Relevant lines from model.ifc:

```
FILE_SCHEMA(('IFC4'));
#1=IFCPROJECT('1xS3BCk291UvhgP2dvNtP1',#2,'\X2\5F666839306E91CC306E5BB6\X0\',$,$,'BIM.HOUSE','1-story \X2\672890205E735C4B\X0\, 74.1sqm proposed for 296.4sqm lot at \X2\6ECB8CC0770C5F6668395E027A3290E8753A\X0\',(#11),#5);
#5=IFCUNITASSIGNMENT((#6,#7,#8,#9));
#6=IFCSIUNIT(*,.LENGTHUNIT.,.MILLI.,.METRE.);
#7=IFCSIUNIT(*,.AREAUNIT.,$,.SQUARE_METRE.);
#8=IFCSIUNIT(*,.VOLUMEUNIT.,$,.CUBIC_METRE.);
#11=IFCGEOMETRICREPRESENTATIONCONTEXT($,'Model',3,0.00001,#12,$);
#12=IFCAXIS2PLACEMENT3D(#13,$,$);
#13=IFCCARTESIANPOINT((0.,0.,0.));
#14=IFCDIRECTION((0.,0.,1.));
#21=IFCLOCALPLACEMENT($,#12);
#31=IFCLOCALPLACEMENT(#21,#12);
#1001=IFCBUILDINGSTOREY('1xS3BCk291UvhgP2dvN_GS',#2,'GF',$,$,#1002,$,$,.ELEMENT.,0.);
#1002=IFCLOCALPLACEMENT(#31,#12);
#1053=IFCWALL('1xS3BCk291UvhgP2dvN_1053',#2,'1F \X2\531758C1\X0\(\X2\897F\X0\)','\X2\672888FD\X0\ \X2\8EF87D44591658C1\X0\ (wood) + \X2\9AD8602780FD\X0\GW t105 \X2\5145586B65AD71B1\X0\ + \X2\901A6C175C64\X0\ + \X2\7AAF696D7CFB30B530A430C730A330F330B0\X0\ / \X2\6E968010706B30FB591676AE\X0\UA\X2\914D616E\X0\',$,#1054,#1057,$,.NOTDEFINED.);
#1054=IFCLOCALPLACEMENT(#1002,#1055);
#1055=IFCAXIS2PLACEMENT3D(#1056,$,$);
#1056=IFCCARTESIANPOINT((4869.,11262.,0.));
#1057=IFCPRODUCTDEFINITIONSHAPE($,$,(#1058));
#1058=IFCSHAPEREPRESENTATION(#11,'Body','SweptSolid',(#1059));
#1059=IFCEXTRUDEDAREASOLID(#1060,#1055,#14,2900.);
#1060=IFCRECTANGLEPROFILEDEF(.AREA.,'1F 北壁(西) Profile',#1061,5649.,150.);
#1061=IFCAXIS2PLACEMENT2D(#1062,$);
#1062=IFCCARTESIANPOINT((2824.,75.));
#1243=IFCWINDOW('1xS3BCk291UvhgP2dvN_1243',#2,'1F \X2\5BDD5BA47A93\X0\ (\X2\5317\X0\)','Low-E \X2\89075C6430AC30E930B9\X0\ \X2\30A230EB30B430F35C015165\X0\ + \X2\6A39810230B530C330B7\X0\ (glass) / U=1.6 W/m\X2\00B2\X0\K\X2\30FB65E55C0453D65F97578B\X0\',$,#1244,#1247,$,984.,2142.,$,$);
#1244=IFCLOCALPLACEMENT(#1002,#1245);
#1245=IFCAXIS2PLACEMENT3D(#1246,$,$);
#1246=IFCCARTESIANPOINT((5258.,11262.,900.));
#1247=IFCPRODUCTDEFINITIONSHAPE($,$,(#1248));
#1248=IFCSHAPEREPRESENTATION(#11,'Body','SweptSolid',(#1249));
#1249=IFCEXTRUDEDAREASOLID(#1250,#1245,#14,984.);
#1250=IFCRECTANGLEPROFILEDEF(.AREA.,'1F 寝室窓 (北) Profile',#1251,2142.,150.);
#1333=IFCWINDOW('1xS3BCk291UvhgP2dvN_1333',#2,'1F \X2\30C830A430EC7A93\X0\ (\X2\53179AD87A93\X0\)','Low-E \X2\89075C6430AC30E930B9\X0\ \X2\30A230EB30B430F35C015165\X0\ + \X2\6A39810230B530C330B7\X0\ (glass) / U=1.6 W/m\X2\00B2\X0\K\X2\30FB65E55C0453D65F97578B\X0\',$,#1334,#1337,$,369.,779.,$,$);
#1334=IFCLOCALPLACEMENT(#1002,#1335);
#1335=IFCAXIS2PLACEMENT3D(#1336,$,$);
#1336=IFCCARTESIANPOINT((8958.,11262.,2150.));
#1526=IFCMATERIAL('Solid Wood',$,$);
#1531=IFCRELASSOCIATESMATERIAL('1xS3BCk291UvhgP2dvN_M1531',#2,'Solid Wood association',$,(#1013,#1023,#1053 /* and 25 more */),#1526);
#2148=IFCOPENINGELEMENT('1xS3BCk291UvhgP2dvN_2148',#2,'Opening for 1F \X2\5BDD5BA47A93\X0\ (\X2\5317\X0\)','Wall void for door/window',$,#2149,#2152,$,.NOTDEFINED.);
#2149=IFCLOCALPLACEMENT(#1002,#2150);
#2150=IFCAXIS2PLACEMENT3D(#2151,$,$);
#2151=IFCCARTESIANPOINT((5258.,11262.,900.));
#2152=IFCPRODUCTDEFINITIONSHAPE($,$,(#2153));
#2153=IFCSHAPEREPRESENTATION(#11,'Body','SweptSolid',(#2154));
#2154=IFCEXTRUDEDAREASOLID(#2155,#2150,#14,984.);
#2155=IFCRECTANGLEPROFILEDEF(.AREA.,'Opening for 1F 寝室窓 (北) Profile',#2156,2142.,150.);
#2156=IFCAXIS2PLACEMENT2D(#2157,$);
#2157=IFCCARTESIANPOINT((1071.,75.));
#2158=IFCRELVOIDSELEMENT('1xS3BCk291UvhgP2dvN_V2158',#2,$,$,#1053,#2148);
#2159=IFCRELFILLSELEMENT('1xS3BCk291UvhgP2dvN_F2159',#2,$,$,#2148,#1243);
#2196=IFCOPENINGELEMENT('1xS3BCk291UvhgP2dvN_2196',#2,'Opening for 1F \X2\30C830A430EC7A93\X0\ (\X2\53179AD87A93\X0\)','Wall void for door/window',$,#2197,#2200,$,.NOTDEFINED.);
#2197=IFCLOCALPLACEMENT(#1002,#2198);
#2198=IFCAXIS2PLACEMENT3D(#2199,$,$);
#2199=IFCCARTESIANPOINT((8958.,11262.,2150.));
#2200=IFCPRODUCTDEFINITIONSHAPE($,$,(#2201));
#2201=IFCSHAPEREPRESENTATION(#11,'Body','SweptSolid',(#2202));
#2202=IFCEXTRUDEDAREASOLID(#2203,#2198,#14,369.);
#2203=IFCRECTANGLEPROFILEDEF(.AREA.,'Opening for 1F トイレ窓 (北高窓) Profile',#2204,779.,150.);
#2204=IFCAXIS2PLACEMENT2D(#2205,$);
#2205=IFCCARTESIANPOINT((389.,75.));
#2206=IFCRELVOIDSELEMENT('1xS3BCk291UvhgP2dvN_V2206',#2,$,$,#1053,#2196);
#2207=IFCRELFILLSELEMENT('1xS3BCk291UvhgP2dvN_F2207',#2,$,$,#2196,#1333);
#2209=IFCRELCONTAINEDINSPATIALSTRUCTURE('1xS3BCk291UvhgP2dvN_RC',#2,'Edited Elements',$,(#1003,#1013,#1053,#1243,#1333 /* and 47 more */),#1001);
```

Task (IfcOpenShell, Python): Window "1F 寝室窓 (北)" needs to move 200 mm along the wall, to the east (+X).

```python
import ifcopenshell
import ifcopenshell.api.geometry
import ifcopenshell.util.placement
import ifcopenshell.util.unit

model = ifcopenshell.open("model.ifc")
unit_scale = ifcopenshell.util.unit.calculate_unit_scale(model)

window = model.by_id(1243)
opening = window.FillsVoids[0].RelatingOpeningElement
wall = opening.VoidsElements[0].RelatingBuildingElement

wall_matrix = ifcopenshell.util.placement.get_local_placement(wall.ObjectPlacement)
shift = wall_matrix[:3, 0] * 0.2 / unit_scale
before = ifcopenshell.util.placement.get_local_placement(window.ObjectPlacement)[:3, 3].copy()

# The window is not placed relative to its opening, so move both.
for product in (opening, window):
    matrix = ifcopenshell.util.placement.get_local_placement(product.ObjectPlacement)
    matrix[:3, 3] += shift
    ifcopenshell.api.geometry.edit_object_placement(model, product=product, matrix=matrix, is_si=False)

after = ifcopenshell.util.placement.get_local_placement(window.ObjectPlacement)[:3, 3]
print("window moved by", (after - before).round(3) + 0.0)

model.write("model_v2.ifc")
```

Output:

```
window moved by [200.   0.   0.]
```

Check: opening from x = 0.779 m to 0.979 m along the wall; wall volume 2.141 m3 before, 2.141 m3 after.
